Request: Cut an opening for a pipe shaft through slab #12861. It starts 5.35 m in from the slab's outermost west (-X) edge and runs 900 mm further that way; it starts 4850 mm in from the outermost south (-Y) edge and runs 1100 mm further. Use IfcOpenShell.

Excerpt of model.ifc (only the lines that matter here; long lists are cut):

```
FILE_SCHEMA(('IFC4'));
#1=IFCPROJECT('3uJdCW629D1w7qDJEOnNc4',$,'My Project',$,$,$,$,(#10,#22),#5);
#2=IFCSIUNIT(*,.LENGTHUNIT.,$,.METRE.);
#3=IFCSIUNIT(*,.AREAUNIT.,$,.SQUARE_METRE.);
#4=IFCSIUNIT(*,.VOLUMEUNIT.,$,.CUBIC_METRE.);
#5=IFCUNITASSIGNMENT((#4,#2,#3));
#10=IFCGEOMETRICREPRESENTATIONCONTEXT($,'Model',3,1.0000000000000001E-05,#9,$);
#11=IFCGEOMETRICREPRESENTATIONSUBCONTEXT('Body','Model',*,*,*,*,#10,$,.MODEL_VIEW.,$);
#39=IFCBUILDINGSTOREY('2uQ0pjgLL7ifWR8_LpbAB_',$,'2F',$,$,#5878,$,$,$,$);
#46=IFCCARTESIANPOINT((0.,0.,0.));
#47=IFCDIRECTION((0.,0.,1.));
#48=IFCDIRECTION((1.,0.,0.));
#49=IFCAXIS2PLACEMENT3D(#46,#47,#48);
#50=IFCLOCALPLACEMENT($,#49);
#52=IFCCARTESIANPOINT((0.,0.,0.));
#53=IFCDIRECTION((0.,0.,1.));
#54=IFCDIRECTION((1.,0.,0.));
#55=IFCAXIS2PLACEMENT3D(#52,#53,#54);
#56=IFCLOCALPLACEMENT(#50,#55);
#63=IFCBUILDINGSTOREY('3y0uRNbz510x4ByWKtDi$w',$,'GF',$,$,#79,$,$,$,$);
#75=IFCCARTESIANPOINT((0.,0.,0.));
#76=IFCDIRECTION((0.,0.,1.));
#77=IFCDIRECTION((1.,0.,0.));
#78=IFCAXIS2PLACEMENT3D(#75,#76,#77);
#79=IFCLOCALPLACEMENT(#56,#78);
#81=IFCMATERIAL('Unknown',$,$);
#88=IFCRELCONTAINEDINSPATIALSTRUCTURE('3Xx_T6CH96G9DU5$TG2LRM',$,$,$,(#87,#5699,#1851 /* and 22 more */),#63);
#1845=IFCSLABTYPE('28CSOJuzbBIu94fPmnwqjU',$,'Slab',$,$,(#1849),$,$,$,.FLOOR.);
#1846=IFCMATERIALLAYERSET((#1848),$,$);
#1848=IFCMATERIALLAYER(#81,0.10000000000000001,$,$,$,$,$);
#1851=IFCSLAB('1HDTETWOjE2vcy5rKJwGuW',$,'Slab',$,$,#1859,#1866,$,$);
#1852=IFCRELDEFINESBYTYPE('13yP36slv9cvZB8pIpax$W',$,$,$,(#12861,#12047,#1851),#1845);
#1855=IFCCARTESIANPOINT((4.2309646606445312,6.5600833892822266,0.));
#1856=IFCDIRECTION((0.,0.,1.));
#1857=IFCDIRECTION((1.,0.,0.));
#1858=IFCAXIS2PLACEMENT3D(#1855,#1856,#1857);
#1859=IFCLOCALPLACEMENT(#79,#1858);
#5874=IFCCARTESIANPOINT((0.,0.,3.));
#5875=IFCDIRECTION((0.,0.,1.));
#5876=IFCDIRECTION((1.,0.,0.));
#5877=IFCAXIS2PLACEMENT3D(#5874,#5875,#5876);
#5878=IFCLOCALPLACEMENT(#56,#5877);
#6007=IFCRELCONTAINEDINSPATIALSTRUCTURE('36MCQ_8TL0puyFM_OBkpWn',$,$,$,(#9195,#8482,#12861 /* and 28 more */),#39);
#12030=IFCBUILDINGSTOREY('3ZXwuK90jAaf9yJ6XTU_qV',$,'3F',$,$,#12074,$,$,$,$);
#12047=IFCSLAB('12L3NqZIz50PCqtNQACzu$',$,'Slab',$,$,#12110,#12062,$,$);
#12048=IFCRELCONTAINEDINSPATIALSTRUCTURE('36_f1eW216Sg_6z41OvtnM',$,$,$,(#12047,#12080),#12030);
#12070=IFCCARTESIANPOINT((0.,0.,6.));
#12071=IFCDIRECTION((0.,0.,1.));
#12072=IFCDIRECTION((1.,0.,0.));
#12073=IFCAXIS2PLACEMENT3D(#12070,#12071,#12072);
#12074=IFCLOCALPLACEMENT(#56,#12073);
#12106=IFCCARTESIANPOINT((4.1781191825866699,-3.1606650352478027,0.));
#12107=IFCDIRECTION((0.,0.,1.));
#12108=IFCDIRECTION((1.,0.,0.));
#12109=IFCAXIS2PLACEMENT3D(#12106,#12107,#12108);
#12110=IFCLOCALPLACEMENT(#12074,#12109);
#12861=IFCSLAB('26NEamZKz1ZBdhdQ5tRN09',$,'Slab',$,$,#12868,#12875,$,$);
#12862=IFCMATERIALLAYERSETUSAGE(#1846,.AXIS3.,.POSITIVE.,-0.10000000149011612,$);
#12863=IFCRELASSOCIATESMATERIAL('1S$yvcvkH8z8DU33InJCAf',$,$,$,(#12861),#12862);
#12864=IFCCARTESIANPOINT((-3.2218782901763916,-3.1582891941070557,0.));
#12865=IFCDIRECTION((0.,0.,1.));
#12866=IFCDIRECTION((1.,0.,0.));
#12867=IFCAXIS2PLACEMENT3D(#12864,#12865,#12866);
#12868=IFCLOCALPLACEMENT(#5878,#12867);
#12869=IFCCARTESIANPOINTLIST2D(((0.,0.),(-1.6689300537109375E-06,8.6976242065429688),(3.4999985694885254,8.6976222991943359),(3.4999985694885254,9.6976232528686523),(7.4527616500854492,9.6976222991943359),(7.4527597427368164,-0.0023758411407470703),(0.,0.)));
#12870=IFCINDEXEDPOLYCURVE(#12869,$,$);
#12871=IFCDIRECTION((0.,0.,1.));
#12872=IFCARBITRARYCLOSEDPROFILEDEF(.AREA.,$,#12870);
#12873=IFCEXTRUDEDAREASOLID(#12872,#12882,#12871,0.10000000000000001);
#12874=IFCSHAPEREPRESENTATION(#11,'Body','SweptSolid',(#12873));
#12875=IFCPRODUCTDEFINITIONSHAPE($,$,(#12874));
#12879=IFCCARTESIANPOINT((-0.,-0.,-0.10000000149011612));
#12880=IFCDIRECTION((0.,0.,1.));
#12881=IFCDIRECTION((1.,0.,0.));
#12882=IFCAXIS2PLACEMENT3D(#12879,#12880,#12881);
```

```python
import numpy as np
import ifcopenshell
import ifcopenshell.api.feature
import ifcopenshell.api.geometry
import ifcopenshell.api.root
import ifcopenshell.geom
import ifcopenshell.util.placement
import ifcopenshell.util.representation
import ifcopenshell.util.shape
import ifcopenshell.util.unit

model = ifcopenshell.open("model.ifc")
unit_scale = ifcopenshell.util.unit.calculate_unit_scale(model)
settings = ifcopenshell.geom.settings()


def volume(element):
    """Net volume in cubic metres, openings subtracted."""
    shape = ifcopenshell.geom.create_shape(settings, element)
    return ifcopenshell.util.shape.get_volume(shape.geometry)


slab = model.by_guid("26NEamZKz1ZBdhdQ5tRN09")
before = volume(slab)

# Extent in the slab's own axes, in metres. The edges named are its -X and -Y sides.
slab_shape = ifcopenshell.geom.create_shape(settings, slab)
vertices = ifcopenshell.util.shape.get_vertices(slab_shape.geometry)
x_min, y_min, bottom = vertices.min(axis=0)
top = vertices[:, 2].max()

opening = ifcopenshell.api.root.create_entity(model, ifc_class="IfcOpeningElement", name="Pipe shaft opening", predefined_type="OPENING")
context = ifcopenshell.util.representation.get_context(model, "Model", "Body", "MODEL_VIEW")
width, depth = 0.9, 1.1
outline = [(0.0, 0.0), (width, 0.0), (width, depth), (0.0, depth), (0.0, 0.0)]
# Overshoot both faces by 50 mm so the cut is clean.
shape = ifcopenshell.api.geometry.add_slab_representation(
    model, context=context, depth=top - bottom + 0.1, polyline=outline
)
ifcopenshell.api.geometry.assign_representation(model, product=opening, representation=shape)

matrix = ifcopenshell.util.placement.get_local_placement(slab.ObjectPlacement)
matrix[:, 3] = matrix @ np.append(np.array([x_min + 5.35, y_min + 4.85, bottom - 0.05]) / unit_scale, 1.0)
ifcopenshell.api.geometry.edit_object_placement(model, product=opening, matrix=matrix, is_si=False)
ifcopenshell.api.feature.add_feature(model, feature=opening, element=slab)

after = volume(slab)

print(f"slab volume {before:.3f} -> {after:.3f} m3")

model.write("model_updated.ifc")
```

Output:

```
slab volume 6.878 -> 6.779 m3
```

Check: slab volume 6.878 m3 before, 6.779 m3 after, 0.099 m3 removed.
